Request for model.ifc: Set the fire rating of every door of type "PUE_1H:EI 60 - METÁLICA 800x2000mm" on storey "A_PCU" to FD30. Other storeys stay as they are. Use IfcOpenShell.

First a look at what the model holds.

```python
import ifcopenshell
import ifcopenshell.util.element

model = ifcopenshell.open("model.ifc")
print(model.schema)
storey = next(s for s in model.by_type("IfcBuildingStorey") if s.Name == "A_PCU")
doors = [e for e in ifcopenshell.util.element.get_decomposition(storey) if e.is_a("IfcDoor")]
seen = {}
for e in doors:
    element_type = ifcopenshell.util.element.get_type(e)
    key = (element_type.Name if element_type != e and element_type else None, ifcopenshell.util.element.get_pset(e, "Pset_DoorCommon", "FireRating"))
    seen[key] = seen.get(key, 0) + 1
for (name, value), count in sorted(seen.items(), key=str):
    print(count, "x", name, "|", value)
```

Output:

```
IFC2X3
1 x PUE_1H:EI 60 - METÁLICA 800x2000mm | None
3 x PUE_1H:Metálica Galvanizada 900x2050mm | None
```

```python
import ifcopenshell
import ifcopenshell.api.pset
import ifcopenshell.util.element

model = ifcopenshell.open("model.ifc")

storey = next(s for s in model.by_type("IfcBuildingStorey") if s.Name == "A_PCU")
doors = [e for e in ifcopenshell.util.element.get_decomposition(storey) if e.is_a("IfcDoor")]

count = 0
for e in doors:
    element_type = ifcopenshell.util.element.get_type(e)
    if element_type in (None, e) or element_type.Name != "PUE_1H:EI 60 - METÁLICA 800x2000mm":
        continue
    # add_pset returns the element's existing set when there is one.
    pset = ifcopenshell.api.pset.add_pset(model, product=e, name="Pset_DoorCommon")
    ifcopenshell.api.pset.edit_pset(model, pset=pset, properties={"FireRating": "FD30"})
    count += 1

print(count, "doors updated")

model.write("model_edited.ifc")
```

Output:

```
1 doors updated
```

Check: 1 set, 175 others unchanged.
